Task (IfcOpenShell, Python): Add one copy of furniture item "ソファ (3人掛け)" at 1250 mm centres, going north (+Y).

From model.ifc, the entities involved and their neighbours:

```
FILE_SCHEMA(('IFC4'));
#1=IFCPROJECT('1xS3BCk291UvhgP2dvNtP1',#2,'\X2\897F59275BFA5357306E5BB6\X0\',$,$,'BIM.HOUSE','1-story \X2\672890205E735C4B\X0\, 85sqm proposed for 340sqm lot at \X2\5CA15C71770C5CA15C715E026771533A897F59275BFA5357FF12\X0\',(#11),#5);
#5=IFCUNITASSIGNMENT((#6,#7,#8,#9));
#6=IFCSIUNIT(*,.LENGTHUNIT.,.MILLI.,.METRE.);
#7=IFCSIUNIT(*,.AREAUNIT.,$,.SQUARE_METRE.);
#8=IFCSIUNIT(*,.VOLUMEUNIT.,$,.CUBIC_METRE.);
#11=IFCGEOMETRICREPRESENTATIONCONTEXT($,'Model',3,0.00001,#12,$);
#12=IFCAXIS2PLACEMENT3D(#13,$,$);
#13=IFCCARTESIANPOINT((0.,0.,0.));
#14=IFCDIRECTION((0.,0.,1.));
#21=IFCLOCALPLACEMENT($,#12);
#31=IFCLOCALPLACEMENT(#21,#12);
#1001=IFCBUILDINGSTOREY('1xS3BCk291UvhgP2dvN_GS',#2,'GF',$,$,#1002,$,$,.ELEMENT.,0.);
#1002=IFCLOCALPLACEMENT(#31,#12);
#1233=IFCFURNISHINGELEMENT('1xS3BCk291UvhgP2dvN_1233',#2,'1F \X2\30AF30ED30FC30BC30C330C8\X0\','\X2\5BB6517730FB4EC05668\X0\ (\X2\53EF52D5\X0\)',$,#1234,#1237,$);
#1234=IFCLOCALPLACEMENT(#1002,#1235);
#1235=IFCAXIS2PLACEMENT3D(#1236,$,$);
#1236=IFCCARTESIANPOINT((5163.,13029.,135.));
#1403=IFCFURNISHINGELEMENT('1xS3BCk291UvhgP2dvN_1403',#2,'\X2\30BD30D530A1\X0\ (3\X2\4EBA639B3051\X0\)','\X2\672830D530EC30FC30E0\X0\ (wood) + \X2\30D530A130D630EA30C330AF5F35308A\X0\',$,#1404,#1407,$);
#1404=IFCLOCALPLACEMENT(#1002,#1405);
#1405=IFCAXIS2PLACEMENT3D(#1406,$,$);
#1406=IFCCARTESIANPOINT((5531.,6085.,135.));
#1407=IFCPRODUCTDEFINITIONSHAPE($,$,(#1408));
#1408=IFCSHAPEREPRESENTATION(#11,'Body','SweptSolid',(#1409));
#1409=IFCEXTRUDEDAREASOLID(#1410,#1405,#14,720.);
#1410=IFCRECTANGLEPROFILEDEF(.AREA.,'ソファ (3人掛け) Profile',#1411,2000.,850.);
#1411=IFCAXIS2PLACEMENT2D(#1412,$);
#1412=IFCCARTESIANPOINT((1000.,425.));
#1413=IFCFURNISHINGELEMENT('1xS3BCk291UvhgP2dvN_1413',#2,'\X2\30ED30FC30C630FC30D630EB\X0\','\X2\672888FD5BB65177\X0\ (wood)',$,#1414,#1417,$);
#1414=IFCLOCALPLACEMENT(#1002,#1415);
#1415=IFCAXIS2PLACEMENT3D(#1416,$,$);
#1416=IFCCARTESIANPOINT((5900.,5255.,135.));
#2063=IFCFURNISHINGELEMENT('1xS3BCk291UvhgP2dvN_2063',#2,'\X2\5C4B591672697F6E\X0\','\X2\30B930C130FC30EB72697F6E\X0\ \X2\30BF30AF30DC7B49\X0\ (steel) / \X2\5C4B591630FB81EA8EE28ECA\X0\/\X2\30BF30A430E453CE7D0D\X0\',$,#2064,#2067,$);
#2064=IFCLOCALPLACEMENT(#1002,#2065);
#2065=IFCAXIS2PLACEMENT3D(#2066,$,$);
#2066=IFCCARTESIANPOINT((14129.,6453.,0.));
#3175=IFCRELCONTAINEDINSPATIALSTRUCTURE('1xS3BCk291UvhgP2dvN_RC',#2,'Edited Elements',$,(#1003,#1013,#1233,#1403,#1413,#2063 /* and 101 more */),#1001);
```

```python
import numpy as np
import ifcopenshell
import ifcopenshell.api.geometry
import ifcopenshell.api.root
import ifcopenshell.util.element
import ifcopenshell.util.placement
import ifcopenshell.util.unit

model = ifcopenshell.open("model.ifc")
unit_scale = ifcopenshell.util.unit.calculate_unit_scale(model)


def reuse_history(source, copy):
    """copy_class also copies each property set's owner history, people and application; keep the originals."""
    for rel in copy.IsDefinedBy:
        if rel.is_a("IfcRelDefinesByProperties") and (history := rel.RelatingPropertyDefinition.OwnerHistory):
            rel.RelatingPropertyDefinition.OwnerHistory = source.OwnerHistory
            ifcopenshell.util.element.remove_deep2(model, history)


source = model.by_id(1403)
base = ifcopenshell.util.placement.get_local_placement(source.ObjectPlacement)
step = np.array([0.0, 1.0, 0.0]) * 1.25 / unit_scale

for i in range(1, 2):
    copy = ifcopenshell.api.root.copy_class(model, product=source)
    copy.Representation = ifcopenshell.util.element.copy_deep(
        model, source.Representation, exclude=["IfcGeometricRepresentationContext", "IfcRepresentationMap"]
    )
    reuse_history(source, copy)
    matrix = base.copy()
    matrix[:3, 3] += i * step
    print("added at", matrix[:3, 3].round(3) + 0.0)
    ifcopenshell.api.geometry.edit_object_placement(model, product=copy, matrix=matrix, is_si=False)

model.write("model_updated.ifc")
```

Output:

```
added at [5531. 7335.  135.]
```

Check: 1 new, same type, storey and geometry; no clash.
